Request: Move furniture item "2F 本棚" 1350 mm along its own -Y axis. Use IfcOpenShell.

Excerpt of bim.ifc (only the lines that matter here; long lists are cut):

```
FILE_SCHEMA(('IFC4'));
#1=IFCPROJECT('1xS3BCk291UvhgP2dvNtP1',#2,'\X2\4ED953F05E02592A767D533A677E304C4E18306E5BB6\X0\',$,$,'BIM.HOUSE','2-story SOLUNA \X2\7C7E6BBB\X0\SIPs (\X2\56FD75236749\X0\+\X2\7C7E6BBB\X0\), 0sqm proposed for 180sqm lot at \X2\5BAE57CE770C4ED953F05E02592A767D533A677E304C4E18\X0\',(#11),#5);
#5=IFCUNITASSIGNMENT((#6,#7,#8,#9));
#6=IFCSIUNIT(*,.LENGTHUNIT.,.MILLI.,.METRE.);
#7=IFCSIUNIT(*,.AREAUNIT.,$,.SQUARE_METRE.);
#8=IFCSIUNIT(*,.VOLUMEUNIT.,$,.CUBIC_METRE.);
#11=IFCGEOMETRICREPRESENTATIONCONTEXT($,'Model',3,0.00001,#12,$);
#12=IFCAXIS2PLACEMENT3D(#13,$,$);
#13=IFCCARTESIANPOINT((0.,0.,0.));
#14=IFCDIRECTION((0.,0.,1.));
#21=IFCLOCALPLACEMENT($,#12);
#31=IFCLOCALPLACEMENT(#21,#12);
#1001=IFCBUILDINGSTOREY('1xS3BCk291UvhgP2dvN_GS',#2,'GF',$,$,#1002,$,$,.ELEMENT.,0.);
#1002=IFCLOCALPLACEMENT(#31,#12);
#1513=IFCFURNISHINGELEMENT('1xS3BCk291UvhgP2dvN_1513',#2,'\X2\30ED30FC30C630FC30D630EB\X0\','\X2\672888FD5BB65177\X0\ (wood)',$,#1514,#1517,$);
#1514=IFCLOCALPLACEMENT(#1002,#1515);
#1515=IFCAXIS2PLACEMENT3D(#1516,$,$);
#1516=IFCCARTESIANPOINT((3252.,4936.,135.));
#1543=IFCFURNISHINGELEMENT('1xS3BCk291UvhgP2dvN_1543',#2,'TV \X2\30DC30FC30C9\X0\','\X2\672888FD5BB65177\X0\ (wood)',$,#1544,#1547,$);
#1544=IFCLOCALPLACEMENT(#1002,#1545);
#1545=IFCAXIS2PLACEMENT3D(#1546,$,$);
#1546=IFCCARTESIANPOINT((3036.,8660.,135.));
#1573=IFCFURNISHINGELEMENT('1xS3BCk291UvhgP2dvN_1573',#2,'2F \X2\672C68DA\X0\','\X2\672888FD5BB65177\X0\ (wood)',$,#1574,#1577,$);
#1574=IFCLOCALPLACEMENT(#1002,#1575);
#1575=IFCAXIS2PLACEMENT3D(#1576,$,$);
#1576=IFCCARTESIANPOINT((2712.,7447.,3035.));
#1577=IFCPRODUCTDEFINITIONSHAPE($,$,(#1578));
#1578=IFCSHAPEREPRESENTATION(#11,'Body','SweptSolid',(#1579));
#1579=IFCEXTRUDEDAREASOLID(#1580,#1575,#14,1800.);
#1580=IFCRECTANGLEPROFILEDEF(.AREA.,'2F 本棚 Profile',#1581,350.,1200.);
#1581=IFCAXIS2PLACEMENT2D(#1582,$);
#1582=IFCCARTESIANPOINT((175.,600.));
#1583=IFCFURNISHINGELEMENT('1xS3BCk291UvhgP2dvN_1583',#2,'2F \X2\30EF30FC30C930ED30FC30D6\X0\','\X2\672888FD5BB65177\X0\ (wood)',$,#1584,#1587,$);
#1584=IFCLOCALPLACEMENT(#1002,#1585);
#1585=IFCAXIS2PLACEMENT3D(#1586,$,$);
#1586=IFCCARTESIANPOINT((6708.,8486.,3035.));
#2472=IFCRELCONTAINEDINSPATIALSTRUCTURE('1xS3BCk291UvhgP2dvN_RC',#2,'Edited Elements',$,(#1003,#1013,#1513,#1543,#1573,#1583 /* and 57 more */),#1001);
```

```python
import ifcopenshell
import ifcopenshell.api.geometry
import ifcopenshell.util.placement
import ifcopenshell.util.unit

model = ifcopenshell.open("bim.ifc")
unit_scale = ifcopenshell.util.unit.calculate_unit_scale(model)

item = model.by_id(1573)
matrix = ifcopenshell.util.placement.get_local_placement(item.ObjectPlacement)
matrix[:3, 3] -= matrix[:3, 1] * 1.35 / unit_scale
ifcopenshell.api.geometry.edit_object_placement(model, product=item, matrix=matrix, is_si=False)

print(ifcopenshell.util.placement.get_local_placement(item.ObjectPlacement).round(3) + 0.0)

model.write("bim_updated.ifc")
```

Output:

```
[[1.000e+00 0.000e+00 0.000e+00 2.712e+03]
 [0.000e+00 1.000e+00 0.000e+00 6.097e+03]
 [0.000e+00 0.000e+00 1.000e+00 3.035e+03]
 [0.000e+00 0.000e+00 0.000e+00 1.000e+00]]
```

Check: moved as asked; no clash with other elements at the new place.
